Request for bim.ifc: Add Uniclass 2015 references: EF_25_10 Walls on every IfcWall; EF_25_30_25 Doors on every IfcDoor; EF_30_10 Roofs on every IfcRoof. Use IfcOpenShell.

First a look at what the model holds.

```python
import ifcopenshell

model = ifcopenshell.open("bim.ifc")
print(model.schema)
print("classifications:", [c.Name for c in model.by_type("IfcClassification")])
for ifc_class in ("IfcDoor", "IfcRoof", "IfcStair", "IfcWall", "IfcWindow"):
    print(ifc_class, len(model.by_type(ifc_class)))
```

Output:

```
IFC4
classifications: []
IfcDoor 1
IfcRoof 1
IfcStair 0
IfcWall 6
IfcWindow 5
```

```python
import ifcopenshell
import ifcopenshell.api.classification

model = ifcopenshell.open("bim.ifc")

system = ifcopenshell.api.classification.add_classification(model, classification="Uniclass 2015")

codes = {
    "IfcWall": ("EF_25_10", "Walls"),
    "IfcDoor": ("EF_25_30_25", "Doors"),
    "IfcRoof": ("EF_30_10", "Roofs"),
}
for ifc_class, (code, name) in codes.items():
    products = model.by_type(ifc_class)
    ifcopenshell.api.classification.add_reference(
        model, products=products, classification=system, identification=code, name=name
    )
    print(code, len(products))

model.write("bim_updated.ifc")
```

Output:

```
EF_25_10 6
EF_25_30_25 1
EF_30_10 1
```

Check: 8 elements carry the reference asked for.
